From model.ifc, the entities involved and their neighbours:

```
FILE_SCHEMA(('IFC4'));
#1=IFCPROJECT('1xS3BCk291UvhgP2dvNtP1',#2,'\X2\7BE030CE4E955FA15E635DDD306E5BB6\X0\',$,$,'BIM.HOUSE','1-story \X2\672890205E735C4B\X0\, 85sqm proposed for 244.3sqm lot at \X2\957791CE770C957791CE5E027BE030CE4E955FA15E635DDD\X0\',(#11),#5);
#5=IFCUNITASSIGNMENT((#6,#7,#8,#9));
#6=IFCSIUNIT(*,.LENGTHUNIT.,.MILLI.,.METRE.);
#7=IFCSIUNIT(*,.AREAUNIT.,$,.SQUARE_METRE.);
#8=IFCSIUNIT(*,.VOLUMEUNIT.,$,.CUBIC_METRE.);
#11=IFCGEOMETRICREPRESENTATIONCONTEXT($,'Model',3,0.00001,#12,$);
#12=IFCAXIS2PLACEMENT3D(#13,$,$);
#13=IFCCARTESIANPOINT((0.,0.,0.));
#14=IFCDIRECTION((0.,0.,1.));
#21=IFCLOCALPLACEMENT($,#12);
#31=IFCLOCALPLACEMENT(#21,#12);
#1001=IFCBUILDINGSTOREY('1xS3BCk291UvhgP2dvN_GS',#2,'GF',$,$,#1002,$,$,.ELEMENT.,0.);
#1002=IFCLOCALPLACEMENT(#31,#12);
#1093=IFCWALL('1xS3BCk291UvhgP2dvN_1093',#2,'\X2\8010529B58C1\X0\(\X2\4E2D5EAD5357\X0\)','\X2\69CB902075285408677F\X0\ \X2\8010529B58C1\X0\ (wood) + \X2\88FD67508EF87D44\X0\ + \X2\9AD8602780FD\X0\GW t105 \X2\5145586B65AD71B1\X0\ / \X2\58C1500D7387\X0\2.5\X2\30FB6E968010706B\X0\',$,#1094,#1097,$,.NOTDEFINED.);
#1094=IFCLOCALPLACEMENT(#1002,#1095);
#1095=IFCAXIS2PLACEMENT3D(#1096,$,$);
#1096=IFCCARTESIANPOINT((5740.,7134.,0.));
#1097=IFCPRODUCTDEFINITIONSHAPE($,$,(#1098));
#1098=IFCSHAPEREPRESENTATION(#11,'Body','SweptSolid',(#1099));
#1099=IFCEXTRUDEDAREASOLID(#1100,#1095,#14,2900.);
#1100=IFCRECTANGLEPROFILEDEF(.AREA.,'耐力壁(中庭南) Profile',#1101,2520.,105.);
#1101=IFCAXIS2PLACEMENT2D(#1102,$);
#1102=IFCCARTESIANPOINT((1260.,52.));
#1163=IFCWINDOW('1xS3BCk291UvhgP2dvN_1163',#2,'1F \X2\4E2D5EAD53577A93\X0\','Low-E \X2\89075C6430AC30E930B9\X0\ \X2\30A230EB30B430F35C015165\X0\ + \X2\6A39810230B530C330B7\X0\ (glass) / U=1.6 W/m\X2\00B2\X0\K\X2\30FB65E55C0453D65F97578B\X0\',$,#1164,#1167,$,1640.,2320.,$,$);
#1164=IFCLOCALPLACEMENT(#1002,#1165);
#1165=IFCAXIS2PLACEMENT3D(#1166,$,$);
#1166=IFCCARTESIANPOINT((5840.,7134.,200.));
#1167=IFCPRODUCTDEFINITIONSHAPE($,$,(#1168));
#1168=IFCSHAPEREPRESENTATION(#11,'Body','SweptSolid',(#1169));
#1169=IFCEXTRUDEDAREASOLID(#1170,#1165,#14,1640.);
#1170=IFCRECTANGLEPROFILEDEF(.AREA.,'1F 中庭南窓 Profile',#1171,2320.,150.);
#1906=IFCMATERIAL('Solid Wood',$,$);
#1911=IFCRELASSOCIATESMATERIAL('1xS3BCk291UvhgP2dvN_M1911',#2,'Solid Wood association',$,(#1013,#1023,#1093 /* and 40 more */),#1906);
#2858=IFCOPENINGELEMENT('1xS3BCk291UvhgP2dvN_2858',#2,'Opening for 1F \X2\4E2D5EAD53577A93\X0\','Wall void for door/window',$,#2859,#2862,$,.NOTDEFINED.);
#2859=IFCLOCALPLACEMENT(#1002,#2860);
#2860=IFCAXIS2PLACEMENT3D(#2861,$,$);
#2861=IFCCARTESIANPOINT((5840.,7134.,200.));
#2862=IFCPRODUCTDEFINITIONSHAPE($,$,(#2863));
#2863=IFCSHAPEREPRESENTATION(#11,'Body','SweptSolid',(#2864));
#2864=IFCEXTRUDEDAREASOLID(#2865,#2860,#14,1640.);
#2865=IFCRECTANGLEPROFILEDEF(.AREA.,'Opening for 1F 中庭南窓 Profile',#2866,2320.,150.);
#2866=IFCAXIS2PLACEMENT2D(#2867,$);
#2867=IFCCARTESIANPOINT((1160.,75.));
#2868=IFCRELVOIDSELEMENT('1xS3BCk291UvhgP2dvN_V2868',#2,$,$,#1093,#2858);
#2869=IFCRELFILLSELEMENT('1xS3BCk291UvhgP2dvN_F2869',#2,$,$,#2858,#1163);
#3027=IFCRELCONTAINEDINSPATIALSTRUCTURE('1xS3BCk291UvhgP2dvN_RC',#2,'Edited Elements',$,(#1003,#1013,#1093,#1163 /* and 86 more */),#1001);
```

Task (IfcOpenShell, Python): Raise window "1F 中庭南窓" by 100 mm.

```python
import numpy as np
import ifcopenshell
import ifcopenshell.api.geometry
import ifcopenshell.util.placement
import ifcopenshell.util.unit

model = ifcopenshell.open("model.ifc")
unit_scale = ifcopenshell.util.unit.calculate_unit_scale(model)

window = model.by_id(1163)
opening = window.FillsVoids[0].RelatingOpeningElement
dz = 0.1 / unit_scale

shift = np.array([0.0, 0.0, dz])
# The window is not placed relative to its opening, so move both.
for product in (opening, window):
    matrix = ifcopenshell.util.placement.get_local_placement(product.ObjectPlacement)
    matrix[:3, 3] += shift
    ifcopenshell.api.geometry.edit_object_placement(model, product=product, matrix=matrix, is_si=False)

print(f"moved by {dz * unit_scale:+.3f} m")

model.write("model_v2.ifc")
```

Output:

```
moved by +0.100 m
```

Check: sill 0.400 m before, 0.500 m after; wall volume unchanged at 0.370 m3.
